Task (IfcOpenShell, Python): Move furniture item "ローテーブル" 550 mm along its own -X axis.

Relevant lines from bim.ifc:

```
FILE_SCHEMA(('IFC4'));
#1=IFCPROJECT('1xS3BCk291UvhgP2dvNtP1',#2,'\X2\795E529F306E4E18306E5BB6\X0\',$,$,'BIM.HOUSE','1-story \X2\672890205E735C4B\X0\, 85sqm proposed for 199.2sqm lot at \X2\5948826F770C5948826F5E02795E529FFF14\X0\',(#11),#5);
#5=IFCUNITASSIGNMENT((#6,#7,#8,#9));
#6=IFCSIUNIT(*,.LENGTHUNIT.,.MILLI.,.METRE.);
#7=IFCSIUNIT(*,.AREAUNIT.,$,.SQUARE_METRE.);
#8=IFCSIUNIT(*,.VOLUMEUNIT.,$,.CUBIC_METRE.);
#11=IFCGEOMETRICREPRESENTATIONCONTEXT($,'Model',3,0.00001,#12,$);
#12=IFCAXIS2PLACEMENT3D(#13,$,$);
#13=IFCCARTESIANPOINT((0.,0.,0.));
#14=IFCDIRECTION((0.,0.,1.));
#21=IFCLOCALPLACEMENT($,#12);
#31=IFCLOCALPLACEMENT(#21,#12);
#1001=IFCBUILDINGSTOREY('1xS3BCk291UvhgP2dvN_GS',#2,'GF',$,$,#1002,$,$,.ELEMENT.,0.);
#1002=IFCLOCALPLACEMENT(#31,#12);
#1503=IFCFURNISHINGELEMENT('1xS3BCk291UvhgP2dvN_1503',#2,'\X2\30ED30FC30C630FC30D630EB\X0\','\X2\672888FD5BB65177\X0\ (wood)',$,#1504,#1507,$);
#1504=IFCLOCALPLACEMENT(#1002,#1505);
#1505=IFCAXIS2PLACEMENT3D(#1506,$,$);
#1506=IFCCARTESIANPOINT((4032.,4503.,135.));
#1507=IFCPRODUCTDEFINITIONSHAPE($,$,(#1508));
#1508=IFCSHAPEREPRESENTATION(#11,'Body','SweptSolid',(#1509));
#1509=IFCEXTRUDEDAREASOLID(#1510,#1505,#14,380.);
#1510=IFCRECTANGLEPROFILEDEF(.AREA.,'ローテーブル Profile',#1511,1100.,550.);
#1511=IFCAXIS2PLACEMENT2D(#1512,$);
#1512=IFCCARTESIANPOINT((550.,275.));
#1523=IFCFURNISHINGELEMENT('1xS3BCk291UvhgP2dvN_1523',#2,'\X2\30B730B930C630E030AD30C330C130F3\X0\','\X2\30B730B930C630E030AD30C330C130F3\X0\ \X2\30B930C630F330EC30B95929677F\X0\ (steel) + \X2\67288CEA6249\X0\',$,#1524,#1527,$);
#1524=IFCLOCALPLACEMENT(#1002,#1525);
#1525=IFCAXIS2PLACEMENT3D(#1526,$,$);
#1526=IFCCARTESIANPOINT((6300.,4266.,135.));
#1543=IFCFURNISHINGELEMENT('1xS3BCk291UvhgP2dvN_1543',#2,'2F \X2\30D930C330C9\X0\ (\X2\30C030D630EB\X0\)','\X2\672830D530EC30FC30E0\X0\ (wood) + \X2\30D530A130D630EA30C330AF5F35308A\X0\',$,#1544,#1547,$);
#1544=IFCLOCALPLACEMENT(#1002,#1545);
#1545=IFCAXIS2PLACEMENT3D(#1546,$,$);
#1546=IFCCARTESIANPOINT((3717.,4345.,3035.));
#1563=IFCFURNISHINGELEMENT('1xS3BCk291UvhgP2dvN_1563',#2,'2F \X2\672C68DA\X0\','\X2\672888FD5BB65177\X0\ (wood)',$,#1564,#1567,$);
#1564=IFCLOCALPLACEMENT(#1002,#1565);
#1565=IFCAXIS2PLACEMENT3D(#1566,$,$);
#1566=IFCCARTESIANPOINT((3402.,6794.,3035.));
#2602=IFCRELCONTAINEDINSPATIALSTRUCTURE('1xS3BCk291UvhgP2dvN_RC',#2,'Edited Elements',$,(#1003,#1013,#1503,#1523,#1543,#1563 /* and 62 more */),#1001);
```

```python
import ifcopenshell
import ifcopenshell.api.geometry
import ifcopenshell.util.placement
import ifcopenshell.util.unit

model = ifcopenshell.open("bim.ifc")
unit_scale = ifcopenshell.util.unit.calculate_unit_scale(model)

item = model.by_guid("1xS3BCk291UvhgP2dvN_1503")
matrix = ifcopenshell.util.placement.get_local_placement(item.ObjectPlacement)
matrix[:3, 3] -= matrix[:3, 0] * 0.55 / unit_scale
ifcopenshell.api.geometry.edit_object_placement(model, product=item, matrix=matrix, is_si=False)

print(ifcopenshell.util.placement.get_local_placement(item.ObjectPlacement).round(3) + 0.0)

model.write("bim_v2.ifc")
```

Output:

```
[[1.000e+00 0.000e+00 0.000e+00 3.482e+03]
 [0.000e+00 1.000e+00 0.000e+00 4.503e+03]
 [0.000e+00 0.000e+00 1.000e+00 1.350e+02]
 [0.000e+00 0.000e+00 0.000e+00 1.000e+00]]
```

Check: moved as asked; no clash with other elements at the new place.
